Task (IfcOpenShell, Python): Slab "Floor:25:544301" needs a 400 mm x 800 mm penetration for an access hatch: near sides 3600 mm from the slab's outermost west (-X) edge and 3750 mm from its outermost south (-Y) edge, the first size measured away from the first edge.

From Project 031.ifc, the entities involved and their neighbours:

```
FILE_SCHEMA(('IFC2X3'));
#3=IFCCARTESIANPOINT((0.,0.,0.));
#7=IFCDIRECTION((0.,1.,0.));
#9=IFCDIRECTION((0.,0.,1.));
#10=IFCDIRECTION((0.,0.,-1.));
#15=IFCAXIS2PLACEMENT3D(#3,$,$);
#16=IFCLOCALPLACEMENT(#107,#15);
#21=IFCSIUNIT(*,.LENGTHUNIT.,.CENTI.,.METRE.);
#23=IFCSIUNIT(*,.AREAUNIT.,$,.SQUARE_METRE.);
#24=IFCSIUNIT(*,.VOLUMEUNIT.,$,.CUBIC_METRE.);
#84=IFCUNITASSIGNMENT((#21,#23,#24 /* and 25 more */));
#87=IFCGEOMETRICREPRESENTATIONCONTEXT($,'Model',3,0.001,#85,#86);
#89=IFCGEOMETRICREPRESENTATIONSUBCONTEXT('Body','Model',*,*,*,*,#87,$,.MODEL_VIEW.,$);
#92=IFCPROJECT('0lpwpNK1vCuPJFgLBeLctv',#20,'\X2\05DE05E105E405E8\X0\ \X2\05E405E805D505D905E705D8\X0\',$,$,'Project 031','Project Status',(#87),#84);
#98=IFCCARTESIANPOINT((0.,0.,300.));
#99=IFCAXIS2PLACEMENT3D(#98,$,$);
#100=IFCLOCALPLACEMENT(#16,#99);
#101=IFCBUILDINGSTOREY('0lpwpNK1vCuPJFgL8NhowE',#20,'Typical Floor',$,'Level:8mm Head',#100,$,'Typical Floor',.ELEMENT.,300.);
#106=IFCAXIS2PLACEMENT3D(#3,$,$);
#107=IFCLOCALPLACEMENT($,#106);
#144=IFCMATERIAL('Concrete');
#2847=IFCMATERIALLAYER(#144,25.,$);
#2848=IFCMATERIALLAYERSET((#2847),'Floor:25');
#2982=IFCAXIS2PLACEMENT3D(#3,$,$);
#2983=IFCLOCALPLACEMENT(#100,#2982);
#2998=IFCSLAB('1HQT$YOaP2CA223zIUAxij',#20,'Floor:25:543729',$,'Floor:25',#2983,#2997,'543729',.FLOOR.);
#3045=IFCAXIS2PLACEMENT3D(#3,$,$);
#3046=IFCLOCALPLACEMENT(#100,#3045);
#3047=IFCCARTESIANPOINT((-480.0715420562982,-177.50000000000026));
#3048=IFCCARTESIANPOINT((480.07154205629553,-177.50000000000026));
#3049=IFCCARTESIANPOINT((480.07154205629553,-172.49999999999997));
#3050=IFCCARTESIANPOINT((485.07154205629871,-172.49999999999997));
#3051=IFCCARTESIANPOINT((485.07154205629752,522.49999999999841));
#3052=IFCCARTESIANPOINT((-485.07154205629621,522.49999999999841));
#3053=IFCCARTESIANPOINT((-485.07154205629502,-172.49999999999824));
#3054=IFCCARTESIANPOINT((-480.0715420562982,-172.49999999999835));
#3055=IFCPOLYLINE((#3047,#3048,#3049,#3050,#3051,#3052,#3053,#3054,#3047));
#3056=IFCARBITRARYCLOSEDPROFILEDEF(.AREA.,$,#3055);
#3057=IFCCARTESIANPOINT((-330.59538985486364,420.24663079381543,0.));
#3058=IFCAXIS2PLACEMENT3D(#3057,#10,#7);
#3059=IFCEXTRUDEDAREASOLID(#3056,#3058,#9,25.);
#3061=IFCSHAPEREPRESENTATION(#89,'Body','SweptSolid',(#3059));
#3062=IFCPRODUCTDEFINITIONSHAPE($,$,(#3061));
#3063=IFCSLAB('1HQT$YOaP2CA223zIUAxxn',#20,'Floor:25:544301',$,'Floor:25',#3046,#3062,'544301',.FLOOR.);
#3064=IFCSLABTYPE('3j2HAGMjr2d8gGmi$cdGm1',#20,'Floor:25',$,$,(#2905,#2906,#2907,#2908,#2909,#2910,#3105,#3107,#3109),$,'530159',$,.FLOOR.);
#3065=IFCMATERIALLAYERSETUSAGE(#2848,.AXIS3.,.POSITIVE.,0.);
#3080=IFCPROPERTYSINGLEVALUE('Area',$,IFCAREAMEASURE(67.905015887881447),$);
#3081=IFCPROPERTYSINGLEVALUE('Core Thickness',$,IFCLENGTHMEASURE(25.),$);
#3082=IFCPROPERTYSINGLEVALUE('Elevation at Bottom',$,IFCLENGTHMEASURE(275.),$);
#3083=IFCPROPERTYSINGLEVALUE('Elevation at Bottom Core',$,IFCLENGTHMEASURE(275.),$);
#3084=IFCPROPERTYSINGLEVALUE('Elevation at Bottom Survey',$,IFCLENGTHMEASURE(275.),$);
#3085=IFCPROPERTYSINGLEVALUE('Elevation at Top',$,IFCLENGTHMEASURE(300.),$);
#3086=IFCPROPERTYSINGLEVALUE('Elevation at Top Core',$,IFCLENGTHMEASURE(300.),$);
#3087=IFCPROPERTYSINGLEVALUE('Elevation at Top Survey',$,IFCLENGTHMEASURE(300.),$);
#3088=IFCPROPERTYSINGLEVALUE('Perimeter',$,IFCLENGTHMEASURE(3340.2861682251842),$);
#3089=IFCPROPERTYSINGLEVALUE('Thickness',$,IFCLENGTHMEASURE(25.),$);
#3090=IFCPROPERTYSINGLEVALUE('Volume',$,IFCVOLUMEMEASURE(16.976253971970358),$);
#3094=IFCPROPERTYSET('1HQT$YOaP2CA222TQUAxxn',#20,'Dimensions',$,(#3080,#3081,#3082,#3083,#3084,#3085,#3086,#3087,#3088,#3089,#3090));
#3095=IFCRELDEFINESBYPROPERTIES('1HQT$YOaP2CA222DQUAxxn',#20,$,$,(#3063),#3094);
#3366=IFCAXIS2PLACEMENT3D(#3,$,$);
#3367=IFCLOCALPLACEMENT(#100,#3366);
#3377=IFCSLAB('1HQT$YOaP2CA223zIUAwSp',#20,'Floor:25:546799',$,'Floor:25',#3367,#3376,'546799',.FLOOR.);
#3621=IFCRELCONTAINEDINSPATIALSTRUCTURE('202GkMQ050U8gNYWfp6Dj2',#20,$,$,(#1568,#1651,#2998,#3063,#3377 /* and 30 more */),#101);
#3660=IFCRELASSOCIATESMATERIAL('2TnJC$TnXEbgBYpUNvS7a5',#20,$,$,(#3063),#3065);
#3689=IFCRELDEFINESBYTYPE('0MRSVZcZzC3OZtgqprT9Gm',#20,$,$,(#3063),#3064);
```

```python
import numpy as np
import ifcopenshell
import ifcopenshell.api.feature
import ifcopenshell.api.geometry
import ifcopenshell.api.pset
import ifcopenshell.api.root
import ifcopenshell.geom
import ifcopenshell.util.element
import ifcopenshell.util.placement
import ifcopenshell.util.representation
import ifcopenshell.util.shape
import ifcopenshell.util.unit

model = ifcopenshell.open("Project 031.ifc")
unit_scale = ifcopenshell.util.unit.calculate_unit_scale(model)
area_scale = ifcopenshell.util.unit.calculate_unit_scale(model, "AREAUNIT")
volume_scale = ifcopenshell.util.unit.calculate_unit_scale(model, "VOLUMEUNIT")
settings = ifcopenshell.geom.settings()


def volume(element):
    """Net volume in cubic metres, openings subtracted."""
    shape = ifcopenshell.geom.create_shape(settings, element)
    return ifcopenshell.util.shape.get_volume(shape.geometry)


slab = model.by_guid("1HQT$YOaP2CA223zIUAxxn")
before = volume(slab)

# Extent in the slab's own axes, in metres. The edges named are its -X and -Y sides.
slab_shape = ifcopenshell.geom.create_shape(settings, slab)
vertices = ifcopenshell.util.shape.get_vertices(slab_shape.geometry)
x_min, y_min, bottom = vertices.min(axis=0)
top = vertices[:, 2].max()

opening = ifcopenshell.api.root.create_entity(model, ifc_class="IfcOpeningElement", name="Access hatch opening")
context = ifcopenshell.util.representation.get_context(model, "Model", "Body", "MODEL_VIEW")
width, depth = 0.4, 0.8
outline = [(0.0, 0.0), (width, 0.0), (width, depth), (0.0, depth), (0.0, 0.0)]
# Overshoot both faces by 50 mm so the cut is clean.
shape = ifcopenshell.api.geometry.add_slab_representation(
    model, context=context, depth=top - bottom + 0.1, polyline=outline
)
ifcopenshell.api.geometry.assign_representation(model, product=opening, representation=shape)

matrix = ifcopenshell.util.placement.get_local_placement(slab.ObjectPlacement)
matrix[:, 3] = matrix @ np.append(np.array([x_min + 3.6, y_min + 3.75, bottom - 0.05]) / unit_scale, 1.0)
ifcopenshell.api.geometry.edit_object_placement(model, product=opening, matrix=matrix, is_si=False)
ifcopenshell.api.feature.add_feature(model, feature=opening, element=slab)

after = volume(slab)

# Update the slab's stored quantities.
pset = model.by_id(ifcopenshell.util.element.get_pset(slab, "Dimensions", should_inherit=False)["id"])
ifcopenshell.api.pset.edit_pset(model, pset=pset, properties={
    "Area": model.create_entity("IfcAreaMeasure", after / (top - bottom) / area_scale),
    "Volume": model.create_entity("IfcVolumeMeasure", after / volume_scale),
})

print(f"slab volume {before:.3f} -> {after:.3f} m3")

model.write("Project 031_edited.ifc")
```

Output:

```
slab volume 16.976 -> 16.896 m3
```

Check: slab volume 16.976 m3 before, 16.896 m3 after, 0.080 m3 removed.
